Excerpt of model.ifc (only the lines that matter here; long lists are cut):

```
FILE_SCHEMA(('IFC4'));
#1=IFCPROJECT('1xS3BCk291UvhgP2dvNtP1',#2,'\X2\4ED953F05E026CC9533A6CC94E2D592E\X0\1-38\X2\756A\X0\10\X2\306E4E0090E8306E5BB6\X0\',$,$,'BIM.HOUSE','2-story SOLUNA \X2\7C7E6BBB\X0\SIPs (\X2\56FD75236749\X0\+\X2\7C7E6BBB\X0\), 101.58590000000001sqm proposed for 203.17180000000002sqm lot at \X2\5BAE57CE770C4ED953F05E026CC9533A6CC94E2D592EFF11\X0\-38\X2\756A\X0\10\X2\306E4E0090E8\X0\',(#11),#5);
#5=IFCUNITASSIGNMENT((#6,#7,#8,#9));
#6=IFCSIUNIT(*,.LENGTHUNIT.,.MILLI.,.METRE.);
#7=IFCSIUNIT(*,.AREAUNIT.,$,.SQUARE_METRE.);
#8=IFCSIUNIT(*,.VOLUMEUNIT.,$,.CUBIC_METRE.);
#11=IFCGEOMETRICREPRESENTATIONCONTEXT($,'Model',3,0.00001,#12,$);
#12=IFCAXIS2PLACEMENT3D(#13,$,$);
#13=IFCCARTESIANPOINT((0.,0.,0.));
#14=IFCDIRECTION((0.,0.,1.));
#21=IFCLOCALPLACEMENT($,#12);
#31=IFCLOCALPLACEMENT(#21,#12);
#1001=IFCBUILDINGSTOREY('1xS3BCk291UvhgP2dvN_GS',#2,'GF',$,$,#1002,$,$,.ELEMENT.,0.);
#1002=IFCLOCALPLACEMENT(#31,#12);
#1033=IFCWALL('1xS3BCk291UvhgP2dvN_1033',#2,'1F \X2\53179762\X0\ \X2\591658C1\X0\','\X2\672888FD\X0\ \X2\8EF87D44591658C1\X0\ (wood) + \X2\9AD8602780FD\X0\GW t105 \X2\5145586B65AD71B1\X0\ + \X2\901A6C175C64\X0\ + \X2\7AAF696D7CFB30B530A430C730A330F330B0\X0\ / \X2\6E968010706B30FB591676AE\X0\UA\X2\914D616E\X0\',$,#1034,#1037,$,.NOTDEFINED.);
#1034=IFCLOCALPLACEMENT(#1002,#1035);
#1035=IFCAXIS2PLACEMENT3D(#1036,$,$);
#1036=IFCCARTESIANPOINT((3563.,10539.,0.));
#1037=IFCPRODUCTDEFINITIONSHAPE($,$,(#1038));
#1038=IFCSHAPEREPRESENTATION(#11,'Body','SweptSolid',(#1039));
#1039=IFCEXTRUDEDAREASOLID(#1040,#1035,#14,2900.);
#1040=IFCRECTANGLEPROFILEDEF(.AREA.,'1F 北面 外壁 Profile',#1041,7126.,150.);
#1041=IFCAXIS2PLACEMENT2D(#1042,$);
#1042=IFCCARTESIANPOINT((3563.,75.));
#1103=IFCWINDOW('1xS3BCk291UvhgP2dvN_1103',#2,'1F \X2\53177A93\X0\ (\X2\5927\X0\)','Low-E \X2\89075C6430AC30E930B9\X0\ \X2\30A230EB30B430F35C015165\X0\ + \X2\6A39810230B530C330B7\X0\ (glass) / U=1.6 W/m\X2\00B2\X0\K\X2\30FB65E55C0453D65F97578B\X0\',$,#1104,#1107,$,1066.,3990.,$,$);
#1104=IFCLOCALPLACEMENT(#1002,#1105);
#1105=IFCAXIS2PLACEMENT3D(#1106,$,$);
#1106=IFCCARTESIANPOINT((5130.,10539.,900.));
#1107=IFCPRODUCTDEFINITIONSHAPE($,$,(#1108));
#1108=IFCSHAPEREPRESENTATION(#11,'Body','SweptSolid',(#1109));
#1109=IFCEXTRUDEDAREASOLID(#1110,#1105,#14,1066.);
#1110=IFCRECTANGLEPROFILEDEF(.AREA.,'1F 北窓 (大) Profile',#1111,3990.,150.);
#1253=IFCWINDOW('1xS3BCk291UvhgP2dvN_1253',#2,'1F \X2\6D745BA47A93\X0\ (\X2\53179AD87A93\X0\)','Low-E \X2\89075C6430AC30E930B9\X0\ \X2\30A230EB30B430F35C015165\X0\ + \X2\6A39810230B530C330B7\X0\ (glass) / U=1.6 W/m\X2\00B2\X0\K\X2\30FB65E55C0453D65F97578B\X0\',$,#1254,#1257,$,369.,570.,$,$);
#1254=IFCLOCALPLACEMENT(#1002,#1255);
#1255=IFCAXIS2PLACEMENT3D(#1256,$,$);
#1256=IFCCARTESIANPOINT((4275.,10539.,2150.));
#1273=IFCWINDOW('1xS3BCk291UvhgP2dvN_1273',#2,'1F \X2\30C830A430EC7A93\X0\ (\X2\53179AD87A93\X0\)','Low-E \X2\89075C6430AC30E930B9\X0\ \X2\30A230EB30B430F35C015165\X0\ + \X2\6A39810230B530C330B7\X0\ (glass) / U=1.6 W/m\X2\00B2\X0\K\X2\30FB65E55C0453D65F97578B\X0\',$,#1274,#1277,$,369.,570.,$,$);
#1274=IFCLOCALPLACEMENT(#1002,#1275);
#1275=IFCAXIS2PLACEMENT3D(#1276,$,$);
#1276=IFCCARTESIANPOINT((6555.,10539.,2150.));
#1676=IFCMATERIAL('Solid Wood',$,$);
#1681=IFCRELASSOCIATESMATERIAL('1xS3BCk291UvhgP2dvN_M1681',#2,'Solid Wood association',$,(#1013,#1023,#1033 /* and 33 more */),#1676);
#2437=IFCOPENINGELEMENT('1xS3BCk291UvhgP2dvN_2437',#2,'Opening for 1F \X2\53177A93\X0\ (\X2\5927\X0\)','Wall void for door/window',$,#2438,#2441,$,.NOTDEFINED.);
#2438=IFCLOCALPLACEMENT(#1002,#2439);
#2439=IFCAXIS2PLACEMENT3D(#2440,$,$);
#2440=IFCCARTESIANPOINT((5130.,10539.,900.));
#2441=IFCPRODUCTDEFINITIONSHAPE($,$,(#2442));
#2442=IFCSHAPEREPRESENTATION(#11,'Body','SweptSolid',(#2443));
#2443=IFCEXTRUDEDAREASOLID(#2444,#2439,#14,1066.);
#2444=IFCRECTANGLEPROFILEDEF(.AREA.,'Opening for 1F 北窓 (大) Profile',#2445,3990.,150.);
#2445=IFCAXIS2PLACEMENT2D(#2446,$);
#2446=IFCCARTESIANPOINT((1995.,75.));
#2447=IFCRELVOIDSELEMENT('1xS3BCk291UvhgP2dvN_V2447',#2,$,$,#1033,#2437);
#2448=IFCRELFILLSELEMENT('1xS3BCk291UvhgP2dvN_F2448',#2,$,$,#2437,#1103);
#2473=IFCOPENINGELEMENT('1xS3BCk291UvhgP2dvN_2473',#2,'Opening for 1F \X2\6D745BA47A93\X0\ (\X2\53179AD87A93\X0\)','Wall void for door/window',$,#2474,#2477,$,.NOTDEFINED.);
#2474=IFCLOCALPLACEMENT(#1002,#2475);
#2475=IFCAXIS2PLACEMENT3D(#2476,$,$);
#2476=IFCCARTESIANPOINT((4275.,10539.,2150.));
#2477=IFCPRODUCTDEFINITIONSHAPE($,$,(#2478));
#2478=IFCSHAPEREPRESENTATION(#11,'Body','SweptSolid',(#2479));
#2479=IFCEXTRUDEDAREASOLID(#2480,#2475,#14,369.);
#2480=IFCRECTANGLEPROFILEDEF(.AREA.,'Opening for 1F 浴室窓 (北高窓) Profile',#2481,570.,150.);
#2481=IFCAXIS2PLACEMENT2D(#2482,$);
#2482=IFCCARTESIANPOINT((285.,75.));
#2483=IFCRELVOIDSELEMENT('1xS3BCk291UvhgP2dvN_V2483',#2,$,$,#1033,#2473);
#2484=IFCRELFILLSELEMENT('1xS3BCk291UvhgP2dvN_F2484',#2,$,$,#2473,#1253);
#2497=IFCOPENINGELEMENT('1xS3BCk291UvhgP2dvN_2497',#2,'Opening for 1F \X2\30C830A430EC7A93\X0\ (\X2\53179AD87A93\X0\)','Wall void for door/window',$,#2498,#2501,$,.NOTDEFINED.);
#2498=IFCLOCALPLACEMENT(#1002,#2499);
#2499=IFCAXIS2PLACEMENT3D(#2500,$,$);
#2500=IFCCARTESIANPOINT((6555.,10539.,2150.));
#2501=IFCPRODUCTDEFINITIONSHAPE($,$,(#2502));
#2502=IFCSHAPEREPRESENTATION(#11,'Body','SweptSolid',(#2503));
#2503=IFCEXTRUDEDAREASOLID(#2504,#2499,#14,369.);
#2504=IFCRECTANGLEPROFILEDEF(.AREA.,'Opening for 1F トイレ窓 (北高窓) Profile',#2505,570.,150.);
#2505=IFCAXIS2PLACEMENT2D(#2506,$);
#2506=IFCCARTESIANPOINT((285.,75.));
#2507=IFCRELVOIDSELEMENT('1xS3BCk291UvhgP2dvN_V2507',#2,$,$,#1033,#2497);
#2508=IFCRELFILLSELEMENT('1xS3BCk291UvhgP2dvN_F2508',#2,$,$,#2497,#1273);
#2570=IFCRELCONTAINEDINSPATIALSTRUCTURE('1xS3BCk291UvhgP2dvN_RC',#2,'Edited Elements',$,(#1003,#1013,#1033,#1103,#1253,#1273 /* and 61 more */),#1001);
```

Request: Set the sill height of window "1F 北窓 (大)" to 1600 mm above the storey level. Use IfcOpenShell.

```python
import numpy as np
import ifcopenshell
import ifcopenshell.api.geometry
import ifcopenshell.geom
import ifcopenshell.util.element
import ifcopenshell.util.placement
import ifcopenshell.util.shape
import ifcopenshell.util.unit

model = ifcopenshell.open("model.ifc")
unit_scale = ifcopenshell.util.unit.calculate_unit_scale(model)

window = model.by_guid("1xS3BCk291UvhgP2dvN_1103")
opening = window.FillsVoids[0].RelatingOpeningElement
storey = ifcopenshell.util.element.get_container(window, ifc_class="IfcBuildingStorey")
level = ifcopenshell.util.placement.get_local_placement(storey.ObjectPlacement)[2, 3]

# The opening's origin need not be at the sill, so measure its lowest point.
shape = ifcopenshell.geom.create_shape(ifcopenshell.geom.settings(), opening)
bottom = ifcopenshell.util.shape.get_shape_bottom_elevation(shape, shape.geometry) / unit_scale
dz = level + 1.6 / unit_scale - bottom

shift = np.array([0.0, 0.0, dz])
# The window is not placed relative to its opening, so move both.
for product in (opening, window):
    matrix = ifcopenshell.util.placement.get_local_placement(product.ObjectPlacement)
    matrix[:3, 3] += shift
    ifcopenshell.api.geometry.edit_object_placement(model, product=product, matrix=matrix, is_si=False)

print(f"moved by {dz * unit_scale:+.3f} m")

model.write("model_updated.ifc")
```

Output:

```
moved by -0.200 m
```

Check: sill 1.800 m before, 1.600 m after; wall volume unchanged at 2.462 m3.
